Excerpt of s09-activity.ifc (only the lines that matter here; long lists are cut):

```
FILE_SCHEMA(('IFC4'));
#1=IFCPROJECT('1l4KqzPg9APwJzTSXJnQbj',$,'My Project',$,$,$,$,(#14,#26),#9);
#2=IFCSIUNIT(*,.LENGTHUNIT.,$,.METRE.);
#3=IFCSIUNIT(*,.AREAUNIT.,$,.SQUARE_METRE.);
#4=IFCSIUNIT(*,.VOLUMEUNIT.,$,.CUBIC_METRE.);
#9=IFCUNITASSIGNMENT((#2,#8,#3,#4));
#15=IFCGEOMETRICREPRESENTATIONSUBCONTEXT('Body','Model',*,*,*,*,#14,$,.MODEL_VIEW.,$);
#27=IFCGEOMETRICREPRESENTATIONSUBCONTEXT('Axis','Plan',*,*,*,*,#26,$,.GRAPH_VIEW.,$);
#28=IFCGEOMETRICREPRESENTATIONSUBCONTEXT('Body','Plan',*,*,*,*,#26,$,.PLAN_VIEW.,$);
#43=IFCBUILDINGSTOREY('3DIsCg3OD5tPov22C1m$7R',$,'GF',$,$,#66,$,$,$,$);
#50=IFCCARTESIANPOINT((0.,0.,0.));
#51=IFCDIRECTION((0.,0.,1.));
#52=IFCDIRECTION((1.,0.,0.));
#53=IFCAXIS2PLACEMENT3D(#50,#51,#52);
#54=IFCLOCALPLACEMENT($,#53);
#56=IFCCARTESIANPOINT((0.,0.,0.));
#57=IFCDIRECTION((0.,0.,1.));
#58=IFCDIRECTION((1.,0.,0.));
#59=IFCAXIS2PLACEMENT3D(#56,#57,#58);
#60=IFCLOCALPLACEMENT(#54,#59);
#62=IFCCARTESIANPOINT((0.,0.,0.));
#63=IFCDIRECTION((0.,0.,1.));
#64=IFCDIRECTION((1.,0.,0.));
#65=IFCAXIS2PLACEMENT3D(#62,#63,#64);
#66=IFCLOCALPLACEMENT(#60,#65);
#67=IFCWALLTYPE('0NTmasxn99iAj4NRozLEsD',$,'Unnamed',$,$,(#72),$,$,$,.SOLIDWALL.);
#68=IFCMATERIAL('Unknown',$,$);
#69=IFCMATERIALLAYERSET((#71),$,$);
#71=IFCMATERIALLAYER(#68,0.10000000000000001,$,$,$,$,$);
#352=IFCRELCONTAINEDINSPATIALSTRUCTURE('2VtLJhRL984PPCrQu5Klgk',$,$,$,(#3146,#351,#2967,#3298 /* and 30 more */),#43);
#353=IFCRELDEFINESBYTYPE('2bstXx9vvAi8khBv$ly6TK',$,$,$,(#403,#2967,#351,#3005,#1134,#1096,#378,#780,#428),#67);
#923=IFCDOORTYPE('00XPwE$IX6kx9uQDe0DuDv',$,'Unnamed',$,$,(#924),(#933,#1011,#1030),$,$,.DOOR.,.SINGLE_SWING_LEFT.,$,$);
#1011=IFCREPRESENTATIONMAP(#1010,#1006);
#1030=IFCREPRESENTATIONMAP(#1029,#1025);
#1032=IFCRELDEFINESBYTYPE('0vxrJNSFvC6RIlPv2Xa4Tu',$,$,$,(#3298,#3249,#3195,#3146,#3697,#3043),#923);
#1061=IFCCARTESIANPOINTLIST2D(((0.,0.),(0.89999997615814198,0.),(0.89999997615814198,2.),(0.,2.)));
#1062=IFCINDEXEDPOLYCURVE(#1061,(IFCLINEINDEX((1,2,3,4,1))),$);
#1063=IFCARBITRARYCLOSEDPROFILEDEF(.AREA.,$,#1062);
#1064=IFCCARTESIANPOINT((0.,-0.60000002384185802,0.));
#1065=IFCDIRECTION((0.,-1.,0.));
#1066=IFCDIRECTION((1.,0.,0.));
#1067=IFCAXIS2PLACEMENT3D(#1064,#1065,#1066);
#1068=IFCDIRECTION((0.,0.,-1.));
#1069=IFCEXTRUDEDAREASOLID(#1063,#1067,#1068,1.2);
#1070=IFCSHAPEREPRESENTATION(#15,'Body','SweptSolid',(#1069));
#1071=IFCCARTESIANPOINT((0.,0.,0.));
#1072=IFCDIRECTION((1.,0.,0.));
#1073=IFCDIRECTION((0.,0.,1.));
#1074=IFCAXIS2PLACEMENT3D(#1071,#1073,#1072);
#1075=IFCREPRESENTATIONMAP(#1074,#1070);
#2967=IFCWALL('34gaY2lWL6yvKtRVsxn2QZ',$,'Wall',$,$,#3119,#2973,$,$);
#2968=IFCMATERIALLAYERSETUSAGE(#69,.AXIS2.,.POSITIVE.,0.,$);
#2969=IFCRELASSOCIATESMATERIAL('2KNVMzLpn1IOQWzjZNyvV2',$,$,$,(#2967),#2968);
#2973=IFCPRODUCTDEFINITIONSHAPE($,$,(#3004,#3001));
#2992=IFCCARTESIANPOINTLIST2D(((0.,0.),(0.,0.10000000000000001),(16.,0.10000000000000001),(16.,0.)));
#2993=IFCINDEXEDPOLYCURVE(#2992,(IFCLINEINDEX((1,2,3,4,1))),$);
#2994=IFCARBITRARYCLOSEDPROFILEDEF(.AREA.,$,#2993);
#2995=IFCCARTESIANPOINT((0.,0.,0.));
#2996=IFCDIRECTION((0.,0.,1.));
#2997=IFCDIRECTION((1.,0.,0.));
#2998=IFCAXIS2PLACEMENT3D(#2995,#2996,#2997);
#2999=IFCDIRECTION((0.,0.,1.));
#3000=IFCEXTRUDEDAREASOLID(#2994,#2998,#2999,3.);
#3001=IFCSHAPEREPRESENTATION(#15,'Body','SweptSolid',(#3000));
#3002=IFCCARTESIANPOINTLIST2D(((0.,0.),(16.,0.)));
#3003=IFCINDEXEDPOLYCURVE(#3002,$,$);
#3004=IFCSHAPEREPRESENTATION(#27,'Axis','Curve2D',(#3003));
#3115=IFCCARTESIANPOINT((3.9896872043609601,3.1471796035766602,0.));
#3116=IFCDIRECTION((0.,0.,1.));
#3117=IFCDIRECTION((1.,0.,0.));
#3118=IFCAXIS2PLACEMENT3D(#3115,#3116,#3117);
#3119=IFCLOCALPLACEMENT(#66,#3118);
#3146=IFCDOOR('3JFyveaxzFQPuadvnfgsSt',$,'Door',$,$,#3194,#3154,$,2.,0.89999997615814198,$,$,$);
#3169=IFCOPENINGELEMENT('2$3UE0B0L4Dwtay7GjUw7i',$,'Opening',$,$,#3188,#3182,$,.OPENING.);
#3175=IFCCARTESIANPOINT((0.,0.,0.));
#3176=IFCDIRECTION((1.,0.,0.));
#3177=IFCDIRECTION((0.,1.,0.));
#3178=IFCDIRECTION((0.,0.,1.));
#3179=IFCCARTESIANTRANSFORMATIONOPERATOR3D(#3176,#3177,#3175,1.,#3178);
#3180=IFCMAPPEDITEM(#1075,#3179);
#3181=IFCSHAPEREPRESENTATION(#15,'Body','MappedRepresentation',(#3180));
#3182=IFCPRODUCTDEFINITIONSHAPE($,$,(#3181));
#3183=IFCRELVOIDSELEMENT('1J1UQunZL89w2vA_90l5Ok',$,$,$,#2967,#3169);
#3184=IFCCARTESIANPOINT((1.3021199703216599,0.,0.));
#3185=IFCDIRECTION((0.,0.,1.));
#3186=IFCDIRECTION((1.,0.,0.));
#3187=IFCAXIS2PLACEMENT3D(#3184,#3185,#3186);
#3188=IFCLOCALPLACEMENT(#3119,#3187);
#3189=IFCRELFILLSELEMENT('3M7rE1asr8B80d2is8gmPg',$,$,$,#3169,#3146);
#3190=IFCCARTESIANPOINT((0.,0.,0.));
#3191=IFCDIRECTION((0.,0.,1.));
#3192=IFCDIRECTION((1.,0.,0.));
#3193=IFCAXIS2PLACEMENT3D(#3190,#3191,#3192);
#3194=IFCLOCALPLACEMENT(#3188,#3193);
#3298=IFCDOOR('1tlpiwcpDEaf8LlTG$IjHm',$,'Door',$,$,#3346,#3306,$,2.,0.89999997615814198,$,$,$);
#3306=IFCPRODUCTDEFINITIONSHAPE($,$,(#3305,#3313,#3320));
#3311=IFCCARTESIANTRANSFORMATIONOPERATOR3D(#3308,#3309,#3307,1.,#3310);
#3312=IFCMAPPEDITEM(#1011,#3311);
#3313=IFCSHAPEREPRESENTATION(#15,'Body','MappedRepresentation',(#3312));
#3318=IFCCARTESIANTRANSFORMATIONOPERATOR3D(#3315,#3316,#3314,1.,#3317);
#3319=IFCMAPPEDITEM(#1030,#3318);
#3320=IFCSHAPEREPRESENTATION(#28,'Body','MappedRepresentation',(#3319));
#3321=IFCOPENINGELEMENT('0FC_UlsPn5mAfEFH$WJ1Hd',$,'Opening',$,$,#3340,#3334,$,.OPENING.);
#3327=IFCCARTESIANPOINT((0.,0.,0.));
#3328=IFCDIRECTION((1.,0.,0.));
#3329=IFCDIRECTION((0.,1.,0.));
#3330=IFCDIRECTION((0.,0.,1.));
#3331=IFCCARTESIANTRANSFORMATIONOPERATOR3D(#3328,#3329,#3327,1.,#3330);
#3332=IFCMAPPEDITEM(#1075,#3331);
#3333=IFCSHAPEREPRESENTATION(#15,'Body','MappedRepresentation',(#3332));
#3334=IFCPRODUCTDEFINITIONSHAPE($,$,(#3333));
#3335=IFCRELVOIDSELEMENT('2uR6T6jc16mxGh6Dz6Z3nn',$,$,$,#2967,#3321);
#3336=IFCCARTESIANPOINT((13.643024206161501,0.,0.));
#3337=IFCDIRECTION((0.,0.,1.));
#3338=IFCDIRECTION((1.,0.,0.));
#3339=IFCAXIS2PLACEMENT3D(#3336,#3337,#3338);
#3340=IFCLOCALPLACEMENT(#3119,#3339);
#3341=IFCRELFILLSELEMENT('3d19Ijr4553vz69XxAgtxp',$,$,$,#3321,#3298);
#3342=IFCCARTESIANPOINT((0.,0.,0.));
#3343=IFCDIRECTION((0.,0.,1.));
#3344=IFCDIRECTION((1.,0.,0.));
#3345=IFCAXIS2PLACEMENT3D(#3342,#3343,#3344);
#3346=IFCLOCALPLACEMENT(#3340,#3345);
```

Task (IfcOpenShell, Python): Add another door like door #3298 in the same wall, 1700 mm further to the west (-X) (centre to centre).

```python
import ifcopenshell
import ifcopenshell.api.feature
import ifcopenshell.api.geometry
import ifcopenshell.api.root
import ifcopenshell.geom
import ifcopenshell.util.element
import ifcopenshell.util.placement
import ifcopenshell.util.shape
import ifcopenshell.util.unit

model = ifcopenshell.open("s09-activity.ifc")
unit_scale = ifcopenshell.util.unit.calculate_unit_scale(model)
settings = ifcopenshell.geom.settings()


def volume(element):
    """Net volume in cubic metres, openings subtracted."""
    shape = ifcopenshell.geom.create_shape(settings, element)
    return ifcopenshell.util.shape.get_volume(shape.geometry)


door = model.by_guid("1tlpiwcpDEaf8LlTG$IjHm")
opening = door.FillsVoids[0].RelatingOpeningElement
wall = opening.VoidsElements[0].RelatingBuildingElement
before = volume(wall)
shift = ifcopenshell.util.placement.get_local_placement(wall.ObjectPlacement)[:3, 0] * -1.7 / unit_scale

# copy_class copies the void relationship, type, container and properties, but no geometry.
new_opening = ifcopenshell.api.root.copy_class(model, product=opening)
new_opening.Representation = ifcopenshell.util.element.copy_deep(
    model, opening.Representation, exclude=["IfcGeometricRepresentationContext", "IfcRepresentationMap"]
)
new_door = ifcopenshell.api.root.copy_class(model, product=door)
new_door.Representation = ifcopenshell.util.element.copy_deep(
    model, door.Representation, exclude=["IfcGeometricRepresentationContext", "IfcRepresentationMap"]
)
ifcopenshell.api.feature.add_filling(model, opening=new_opening, element=new_door)

for old, new in ((opening, new_opening), (door, new_door)):
    matrix = ifcopenshell.util.placement.get_local_placement(old.ObjectPlacement)
    matrix[:3, 3] += shift
    ifcopenshell.api.geometry.edit_object_placement(model, product=new, matrix=matrix, is_si=False)

after = volume(wall)

print(f"wall volume {before:.3f} -> {after:.3f} m3")

model.write("s09-activity_edited.ifc")
```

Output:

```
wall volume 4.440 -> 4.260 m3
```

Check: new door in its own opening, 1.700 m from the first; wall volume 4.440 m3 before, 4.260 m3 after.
